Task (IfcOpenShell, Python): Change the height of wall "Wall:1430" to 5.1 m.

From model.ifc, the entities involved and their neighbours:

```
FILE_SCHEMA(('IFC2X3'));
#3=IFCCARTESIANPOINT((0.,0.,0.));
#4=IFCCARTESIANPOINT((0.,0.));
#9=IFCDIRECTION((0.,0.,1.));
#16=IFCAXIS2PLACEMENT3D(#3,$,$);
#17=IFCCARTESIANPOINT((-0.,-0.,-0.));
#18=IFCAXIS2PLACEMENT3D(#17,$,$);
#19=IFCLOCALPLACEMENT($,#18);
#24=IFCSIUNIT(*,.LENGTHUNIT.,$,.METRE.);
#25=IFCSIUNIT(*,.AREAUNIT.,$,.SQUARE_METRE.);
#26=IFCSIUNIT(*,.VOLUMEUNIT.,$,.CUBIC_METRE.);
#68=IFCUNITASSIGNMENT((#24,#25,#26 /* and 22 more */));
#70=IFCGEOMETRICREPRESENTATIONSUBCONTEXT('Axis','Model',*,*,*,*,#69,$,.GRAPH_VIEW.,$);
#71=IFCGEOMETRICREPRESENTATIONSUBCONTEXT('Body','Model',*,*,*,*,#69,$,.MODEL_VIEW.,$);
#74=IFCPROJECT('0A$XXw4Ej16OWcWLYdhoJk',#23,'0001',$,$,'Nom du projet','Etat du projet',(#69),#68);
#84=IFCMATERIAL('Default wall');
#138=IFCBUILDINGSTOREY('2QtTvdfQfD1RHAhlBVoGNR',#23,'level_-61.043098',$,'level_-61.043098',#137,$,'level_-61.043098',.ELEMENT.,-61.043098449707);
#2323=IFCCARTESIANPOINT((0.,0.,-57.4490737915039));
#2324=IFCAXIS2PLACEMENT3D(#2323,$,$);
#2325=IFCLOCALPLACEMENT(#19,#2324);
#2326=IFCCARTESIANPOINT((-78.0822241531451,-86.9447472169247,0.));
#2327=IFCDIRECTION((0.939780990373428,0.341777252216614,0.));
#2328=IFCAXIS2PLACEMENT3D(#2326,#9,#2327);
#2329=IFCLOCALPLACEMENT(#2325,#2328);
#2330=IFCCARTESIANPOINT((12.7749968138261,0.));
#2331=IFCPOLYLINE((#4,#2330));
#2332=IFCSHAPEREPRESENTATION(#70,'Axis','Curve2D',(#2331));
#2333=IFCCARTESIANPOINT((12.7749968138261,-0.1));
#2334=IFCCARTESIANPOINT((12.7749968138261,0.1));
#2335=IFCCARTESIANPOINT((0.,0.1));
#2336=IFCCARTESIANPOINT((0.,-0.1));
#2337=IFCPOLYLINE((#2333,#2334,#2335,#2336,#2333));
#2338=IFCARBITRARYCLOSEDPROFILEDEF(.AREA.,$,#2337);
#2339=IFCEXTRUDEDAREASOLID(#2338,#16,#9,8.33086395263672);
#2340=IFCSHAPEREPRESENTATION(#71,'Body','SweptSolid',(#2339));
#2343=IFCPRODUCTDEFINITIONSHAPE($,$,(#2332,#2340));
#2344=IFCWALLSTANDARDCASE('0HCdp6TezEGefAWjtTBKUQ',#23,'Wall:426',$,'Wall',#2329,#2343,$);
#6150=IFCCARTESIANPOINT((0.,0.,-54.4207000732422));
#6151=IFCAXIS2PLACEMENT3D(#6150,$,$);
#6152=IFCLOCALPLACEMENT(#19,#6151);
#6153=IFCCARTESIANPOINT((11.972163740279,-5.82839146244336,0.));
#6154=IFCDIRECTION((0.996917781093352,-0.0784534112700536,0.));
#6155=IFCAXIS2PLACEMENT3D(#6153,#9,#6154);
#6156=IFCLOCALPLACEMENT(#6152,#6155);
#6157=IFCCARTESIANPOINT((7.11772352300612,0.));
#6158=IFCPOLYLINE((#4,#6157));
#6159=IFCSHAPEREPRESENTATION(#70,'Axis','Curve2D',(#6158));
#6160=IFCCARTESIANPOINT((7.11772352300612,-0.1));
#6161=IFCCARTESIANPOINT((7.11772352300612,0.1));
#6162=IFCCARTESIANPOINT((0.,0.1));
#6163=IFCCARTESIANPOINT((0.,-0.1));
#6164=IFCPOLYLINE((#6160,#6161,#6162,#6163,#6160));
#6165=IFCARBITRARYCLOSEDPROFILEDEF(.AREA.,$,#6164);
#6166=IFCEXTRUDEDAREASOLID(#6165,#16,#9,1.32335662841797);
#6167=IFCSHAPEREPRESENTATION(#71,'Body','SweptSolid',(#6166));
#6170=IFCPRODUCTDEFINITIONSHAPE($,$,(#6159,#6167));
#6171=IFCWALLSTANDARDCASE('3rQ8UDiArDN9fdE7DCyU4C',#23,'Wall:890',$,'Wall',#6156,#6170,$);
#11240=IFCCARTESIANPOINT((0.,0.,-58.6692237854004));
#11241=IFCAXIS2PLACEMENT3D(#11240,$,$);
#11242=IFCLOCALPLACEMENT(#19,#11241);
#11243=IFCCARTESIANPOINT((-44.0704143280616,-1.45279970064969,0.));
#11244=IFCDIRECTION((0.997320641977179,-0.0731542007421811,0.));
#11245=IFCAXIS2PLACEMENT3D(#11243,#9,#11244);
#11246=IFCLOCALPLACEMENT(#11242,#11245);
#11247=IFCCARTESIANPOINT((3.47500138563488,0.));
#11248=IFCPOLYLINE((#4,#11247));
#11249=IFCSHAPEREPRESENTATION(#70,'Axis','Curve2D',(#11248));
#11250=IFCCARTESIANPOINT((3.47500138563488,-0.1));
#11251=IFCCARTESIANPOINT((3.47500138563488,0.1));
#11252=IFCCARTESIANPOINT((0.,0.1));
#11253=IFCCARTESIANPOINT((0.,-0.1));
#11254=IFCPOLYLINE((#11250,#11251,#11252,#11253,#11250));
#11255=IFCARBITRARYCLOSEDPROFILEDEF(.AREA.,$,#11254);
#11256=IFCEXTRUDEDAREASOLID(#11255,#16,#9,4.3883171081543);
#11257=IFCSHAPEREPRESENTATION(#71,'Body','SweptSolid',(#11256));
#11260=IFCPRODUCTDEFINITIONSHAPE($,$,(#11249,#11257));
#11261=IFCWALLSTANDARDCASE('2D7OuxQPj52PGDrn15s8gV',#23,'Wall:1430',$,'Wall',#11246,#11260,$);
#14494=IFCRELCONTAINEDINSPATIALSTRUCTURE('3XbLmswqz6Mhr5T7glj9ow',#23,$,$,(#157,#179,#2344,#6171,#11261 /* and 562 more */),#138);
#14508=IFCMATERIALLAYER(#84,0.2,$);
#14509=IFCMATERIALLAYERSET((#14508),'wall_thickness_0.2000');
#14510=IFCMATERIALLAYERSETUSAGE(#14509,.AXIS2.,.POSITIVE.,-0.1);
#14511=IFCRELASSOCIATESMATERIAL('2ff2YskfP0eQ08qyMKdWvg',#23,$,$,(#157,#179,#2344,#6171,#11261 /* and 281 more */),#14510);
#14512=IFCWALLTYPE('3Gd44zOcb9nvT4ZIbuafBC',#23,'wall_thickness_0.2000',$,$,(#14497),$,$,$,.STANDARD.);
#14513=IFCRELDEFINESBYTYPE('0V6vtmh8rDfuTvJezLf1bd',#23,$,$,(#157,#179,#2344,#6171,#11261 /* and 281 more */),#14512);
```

```python
import ifcopenshell
import ifcopenshell.geom
import ifcopenshell.util.representation
import ifcopenshell.util.shape
import ifcopenshell.util.unit

model = ifcopenshell.open("model.ifc")
unit_scale = ifcopenshell.util.unit.calculate_unit_scale(model)
settings = ifcopenshell.geom.settings()


def volume(element):
    """Net volume in cubic metres, openings subtracted."""
    shape = ifcopenshell.geom.create_shape(settings, element)
    return ifcopenshell.util.shape.get_volume(shape.geometry)


wall = model.by_id(11261)
before = volume(wall)

body = ifcopenshell.util.representation.get_representation(wall, "Model", "Body")
solid = body.Items[0]
old_height = solid.Depth
solid.Depth = 5.1 / unit_scale
after = volume(wall)

print(f"height {old_height:g} -> {solid.Depth:g}, volume {before:.3f} -> {after:.3f} m3")

model.write("model_v2.ifc")
```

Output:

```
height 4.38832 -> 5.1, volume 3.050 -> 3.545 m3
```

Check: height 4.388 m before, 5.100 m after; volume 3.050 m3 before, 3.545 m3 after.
